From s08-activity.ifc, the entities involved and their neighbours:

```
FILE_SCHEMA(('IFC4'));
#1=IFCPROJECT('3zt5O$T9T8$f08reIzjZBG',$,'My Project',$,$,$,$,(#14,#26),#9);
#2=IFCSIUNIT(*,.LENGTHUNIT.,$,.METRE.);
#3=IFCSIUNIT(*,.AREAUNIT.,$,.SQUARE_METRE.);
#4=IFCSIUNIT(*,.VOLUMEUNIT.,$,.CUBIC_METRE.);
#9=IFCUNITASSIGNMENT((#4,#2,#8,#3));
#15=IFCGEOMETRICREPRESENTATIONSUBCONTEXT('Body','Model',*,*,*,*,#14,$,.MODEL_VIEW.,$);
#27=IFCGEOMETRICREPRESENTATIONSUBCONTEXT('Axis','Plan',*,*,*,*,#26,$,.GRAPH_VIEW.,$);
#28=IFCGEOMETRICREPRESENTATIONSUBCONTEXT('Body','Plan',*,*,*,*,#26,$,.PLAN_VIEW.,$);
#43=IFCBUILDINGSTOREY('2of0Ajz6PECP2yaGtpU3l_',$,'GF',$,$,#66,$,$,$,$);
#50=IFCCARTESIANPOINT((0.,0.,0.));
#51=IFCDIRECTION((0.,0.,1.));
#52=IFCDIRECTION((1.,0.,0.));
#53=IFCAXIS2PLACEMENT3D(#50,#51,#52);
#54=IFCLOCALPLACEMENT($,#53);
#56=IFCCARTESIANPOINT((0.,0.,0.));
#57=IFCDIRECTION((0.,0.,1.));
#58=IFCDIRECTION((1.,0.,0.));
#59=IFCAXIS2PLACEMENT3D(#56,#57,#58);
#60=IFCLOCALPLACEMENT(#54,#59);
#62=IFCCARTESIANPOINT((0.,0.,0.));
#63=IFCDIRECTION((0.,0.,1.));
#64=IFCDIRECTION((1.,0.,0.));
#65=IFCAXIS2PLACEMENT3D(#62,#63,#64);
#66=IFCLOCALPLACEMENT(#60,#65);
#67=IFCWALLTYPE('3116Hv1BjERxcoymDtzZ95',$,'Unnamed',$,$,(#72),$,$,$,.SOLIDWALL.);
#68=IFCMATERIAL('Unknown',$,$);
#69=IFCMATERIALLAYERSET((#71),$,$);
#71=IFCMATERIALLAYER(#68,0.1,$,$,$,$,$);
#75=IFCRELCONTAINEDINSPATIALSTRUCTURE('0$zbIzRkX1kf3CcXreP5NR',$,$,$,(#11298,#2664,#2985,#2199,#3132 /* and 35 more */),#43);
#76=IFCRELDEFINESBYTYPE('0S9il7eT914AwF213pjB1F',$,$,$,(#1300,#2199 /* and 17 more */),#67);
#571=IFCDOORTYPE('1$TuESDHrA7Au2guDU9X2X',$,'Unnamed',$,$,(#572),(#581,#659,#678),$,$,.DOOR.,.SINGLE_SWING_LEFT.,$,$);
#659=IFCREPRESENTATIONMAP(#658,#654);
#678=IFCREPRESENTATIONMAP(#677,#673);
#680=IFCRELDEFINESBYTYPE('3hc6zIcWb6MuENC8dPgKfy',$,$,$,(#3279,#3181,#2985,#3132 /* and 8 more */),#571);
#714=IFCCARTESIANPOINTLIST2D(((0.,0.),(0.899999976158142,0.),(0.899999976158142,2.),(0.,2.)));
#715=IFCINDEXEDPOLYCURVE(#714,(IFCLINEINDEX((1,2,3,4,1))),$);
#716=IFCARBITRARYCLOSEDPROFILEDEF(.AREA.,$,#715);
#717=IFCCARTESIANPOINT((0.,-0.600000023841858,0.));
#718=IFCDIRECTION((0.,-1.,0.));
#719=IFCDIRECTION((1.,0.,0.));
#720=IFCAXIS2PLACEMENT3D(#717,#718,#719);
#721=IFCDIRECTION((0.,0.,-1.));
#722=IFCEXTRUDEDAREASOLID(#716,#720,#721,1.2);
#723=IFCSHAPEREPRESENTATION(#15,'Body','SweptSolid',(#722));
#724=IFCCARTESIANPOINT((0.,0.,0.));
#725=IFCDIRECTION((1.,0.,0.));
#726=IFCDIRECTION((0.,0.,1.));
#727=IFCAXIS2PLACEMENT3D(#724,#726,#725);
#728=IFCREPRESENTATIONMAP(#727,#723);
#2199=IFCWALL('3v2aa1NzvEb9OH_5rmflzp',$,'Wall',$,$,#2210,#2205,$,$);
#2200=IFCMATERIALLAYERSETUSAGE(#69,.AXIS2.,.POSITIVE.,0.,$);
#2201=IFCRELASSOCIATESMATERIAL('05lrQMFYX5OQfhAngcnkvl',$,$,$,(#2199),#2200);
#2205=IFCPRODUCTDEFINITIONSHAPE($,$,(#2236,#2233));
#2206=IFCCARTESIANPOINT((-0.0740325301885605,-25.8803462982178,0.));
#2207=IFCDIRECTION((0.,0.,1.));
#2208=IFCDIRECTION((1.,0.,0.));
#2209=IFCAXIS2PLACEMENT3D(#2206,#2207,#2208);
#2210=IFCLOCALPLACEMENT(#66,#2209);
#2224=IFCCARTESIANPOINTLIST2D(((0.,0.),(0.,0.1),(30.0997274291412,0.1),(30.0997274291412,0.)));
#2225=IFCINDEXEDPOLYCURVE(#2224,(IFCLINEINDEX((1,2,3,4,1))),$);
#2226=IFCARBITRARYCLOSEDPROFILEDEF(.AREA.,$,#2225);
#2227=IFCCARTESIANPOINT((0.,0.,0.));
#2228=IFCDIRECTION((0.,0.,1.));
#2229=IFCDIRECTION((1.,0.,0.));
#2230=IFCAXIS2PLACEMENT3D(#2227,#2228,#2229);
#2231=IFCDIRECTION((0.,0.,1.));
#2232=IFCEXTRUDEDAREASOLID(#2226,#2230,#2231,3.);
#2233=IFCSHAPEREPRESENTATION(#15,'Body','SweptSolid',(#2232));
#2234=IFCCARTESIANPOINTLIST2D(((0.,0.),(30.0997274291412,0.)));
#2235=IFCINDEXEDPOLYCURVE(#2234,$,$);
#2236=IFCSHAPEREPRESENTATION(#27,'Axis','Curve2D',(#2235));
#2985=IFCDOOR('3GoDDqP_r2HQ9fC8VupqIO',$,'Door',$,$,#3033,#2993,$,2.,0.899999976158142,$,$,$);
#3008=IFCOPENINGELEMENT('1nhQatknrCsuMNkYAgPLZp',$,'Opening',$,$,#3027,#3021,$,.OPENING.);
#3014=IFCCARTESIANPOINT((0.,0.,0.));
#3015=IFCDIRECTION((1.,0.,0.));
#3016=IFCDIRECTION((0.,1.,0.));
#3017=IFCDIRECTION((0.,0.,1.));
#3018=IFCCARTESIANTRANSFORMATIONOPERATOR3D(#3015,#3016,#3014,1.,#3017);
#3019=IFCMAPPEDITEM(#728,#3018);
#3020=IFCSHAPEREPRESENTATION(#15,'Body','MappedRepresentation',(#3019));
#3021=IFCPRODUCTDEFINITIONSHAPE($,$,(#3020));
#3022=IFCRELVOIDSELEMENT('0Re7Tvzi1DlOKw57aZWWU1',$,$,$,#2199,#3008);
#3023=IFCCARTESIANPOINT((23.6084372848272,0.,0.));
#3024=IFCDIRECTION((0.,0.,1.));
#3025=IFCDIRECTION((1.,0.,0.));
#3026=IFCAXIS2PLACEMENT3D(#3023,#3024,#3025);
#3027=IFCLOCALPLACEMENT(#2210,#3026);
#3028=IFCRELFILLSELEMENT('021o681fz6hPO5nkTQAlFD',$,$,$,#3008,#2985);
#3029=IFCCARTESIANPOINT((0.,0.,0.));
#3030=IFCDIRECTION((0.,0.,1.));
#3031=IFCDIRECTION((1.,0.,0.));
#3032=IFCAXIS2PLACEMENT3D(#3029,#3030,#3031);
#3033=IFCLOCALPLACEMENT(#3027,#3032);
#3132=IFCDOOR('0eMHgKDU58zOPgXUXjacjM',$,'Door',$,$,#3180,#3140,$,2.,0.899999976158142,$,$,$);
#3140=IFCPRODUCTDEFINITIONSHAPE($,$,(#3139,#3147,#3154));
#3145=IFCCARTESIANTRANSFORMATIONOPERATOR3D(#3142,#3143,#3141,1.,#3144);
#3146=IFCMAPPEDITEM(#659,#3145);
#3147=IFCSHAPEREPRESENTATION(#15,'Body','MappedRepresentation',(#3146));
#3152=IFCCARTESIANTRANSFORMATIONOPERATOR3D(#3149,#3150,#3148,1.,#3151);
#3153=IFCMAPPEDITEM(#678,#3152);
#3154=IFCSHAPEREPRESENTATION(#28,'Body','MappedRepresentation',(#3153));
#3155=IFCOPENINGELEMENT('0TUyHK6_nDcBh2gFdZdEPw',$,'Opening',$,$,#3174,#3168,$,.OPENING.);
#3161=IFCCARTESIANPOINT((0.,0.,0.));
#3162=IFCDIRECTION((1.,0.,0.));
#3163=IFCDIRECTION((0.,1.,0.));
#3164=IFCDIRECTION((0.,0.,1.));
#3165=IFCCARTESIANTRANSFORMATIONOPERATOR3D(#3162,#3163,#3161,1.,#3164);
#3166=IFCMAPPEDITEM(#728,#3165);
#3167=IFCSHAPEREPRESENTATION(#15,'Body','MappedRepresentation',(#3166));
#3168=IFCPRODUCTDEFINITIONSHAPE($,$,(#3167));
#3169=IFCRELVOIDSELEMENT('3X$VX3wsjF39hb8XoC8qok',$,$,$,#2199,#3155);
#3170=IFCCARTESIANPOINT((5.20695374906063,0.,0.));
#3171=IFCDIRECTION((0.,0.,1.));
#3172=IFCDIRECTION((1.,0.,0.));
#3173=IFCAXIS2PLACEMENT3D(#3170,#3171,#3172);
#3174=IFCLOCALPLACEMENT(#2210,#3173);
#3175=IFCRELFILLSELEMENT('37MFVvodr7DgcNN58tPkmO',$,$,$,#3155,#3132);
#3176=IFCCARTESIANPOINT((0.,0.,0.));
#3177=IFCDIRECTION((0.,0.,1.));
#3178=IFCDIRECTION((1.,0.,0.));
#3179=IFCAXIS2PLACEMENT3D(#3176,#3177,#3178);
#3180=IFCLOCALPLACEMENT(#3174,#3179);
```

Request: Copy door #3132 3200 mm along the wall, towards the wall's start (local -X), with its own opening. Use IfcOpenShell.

```python
import ifcopenshell
import ifcopenshell.api.feature
import ifcopenshell.api.geometry
import ifcopenshell.api.root
import ifcopenshell.geom
import ifcopenshell.util.element
import ifcopenshell.util.placement
import ifcopenshell.util.shape

model = ifcopenshell.open("s08-activity.ifc")
settings = ifcopenshell.geom.settings()


def volume(element):
    """Net volume in cubic metres, openings subtracted."""
    shape = ifcopenshell.geom.create_shape(settings, element)
    return ifcopenshell.util.shape.get_volume(shape.geometry)


door = model.by_guid("0eMHgKDU58zOPgXUXjacjM")
opening = door.FillsVoids[0].RelatingOpeningElement
wall = opening.VoidsElements[0].RelatingBuildingElement
before = volume(wall)
shift = ifcopenshell.util.placement.get_local_placement(wall.ObjectPlacement)[:3, 0] * -3.2

# copy_class copies the void relationship, type, container and properties, but no geometry.
new_opening = ifcopenshell.api.root.copy_class(model, product=opening)
new_opening.Representation = ifcopenshell.util.element.copy_deep(
    model, opening.Representation, exclude=["IfcGeometricRepresentationContext", "IfcRepresentationMap"]
)
new_door = ifcopenshell.api.root.copy_class(model, product=door)
new_door.Representation = ifcopenshell.util.element.copy_deep(
    model, door.Representation, exclude=["IfcGeometricRepresentationContext", "IfcRepresentationMap"]
)
ifcopenshell.api.feature.add_filling(model, opening=new_opening, element=new_door)

for old, new in ((opening, new_opening), (door, new_door)):
    matrix = ifcopenshell.util.placement.get_local_placement(old.ObjectPlacement)
    matrix[:3, 3] += shift
    ifcopenshell.api.geometry.edit_object_placement(model, product=new, matrix=matrix, is_si=False)

after = volume(wall)

print(f"wall volume {before:.3f} -> {after:.3f} m3")

model.write("s08-activity_edited.ifc")
```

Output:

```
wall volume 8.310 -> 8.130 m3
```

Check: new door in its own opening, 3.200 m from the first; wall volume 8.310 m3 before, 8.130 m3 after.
